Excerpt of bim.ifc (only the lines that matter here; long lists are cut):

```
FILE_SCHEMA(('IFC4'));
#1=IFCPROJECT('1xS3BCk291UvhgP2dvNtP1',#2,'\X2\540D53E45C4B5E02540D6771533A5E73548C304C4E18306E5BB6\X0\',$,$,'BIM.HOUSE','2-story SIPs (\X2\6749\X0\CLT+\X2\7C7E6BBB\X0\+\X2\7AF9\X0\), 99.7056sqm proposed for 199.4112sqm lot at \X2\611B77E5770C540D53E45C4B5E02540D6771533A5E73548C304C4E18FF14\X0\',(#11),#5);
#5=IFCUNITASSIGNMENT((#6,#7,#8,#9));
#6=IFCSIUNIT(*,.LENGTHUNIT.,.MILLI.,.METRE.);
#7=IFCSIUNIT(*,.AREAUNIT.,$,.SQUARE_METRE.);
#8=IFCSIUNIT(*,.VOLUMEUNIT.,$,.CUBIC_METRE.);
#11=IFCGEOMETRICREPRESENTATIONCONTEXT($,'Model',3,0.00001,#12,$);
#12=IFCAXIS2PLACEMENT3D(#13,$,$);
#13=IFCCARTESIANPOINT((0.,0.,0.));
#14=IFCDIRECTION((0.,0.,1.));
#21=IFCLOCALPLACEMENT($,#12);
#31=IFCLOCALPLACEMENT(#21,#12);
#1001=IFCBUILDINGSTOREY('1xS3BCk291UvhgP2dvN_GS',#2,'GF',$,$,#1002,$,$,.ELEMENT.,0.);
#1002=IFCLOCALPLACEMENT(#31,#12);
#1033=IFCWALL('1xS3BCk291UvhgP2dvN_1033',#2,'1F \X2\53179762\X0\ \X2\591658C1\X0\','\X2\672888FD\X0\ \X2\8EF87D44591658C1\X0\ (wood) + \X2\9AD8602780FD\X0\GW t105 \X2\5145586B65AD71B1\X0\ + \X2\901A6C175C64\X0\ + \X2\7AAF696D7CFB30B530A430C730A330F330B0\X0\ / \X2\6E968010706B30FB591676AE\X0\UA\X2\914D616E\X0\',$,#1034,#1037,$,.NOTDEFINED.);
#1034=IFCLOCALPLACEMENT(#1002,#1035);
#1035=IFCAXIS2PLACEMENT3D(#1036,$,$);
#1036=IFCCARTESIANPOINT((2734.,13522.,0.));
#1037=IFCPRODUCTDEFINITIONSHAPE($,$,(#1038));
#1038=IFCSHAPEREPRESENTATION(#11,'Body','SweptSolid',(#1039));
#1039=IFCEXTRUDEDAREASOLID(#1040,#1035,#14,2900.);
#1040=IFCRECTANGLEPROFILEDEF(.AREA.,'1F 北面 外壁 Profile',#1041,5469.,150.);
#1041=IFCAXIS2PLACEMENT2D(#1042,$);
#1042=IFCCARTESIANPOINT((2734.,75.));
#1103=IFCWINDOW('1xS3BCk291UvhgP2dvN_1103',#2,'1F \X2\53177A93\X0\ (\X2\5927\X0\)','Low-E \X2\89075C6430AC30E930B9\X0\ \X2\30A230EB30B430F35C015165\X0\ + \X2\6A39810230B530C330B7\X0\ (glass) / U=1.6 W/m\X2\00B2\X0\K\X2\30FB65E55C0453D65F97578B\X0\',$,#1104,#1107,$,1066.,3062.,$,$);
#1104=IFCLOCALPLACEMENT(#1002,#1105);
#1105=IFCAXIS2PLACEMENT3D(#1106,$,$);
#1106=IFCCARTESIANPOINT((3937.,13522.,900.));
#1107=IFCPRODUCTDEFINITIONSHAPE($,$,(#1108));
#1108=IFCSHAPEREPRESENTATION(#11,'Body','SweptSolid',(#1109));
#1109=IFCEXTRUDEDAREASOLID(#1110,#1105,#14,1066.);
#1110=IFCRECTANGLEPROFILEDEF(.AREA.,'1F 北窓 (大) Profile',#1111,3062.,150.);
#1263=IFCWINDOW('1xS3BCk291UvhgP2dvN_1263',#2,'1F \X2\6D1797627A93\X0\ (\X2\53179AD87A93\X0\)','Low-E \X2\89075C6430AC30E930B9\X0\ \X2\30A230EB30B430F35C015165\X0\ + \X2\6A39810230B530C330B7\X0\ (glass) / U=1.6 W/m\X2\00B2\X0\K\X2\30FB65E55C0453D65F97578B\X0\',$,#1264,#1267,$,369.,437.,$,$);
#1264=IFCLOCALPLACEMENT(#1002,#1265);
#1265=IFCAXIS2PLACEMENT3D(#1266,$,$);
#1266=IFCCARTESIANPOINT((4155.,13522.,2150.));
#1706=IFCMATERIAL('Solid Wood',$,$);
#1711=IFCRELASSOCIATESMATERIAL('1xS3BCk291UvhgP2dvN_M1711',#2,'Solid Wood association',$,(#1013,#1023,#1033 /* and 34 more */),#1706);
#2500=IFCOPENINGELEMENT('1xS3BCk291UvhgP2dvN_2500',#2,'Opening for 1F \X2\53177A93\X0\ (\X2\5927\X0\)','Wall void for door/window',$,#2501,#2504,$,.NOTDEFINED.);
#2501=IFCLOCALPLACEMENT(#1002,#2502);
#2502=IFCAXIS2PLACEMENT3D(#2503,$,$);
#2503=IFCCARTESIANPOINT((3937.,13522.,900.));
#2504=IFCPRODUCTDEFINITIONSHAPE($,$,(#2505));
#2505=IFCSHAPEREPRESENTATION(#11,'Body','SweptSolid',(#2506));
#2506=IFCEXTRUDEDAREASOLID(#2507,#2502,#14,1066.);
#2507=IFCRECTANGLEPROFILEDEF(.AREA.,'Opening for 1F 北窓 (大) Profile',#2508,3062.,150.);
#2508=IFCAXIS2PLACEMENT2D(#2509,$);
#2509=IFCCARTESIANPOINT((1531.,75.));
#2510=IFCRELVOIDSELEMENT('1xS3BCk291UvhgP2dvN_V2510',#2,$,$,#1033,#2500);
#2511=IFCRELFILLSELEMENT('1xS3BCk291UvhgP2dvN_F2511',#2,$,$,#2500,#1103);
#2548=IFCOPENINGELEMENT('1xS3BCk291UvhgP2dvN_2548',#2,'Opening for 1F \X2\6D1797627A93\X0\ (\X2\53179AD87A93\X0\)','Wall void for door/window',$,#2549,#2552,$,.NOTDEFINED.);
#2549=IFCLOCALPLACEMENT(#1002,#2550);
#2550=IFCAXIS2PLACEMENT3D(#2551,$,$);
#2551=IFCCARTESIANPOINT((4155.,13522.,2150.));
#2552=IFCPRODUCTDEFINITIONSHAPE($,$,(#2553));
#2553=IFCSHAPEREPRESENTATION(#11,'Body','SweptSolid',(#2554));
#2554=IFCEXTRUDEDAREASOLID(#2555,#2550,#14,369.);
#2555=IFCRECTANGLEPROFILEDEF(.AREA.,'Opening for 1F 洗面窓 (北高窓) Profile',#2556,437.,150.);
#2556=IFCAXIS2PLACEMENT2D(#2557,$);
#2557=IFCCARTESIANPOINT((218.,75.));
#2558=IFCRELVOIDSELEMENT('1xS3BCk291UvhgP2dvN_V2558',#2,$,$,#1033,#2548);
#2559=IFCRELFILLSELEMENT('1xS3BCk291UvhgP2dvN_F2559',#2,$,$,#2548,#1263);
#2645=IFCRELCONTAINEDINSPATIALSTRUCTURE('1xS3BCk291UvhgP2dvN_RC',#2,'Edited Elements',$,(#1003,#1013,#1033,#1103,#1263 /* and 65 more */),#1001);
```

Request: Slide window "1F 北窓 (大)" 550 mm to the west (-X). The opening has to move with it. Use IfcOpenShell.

```python
import ifcopenshell
import ifcopenshell.api.geometry
import ifcopenshell.util.placement

model = ifcopenshell.open("bim.ifc")

window = model.by_guid("1xS3BCk291UvhgP2dvN_1103")
opening = window.FillsVoids[0].RelatingOpeningElement
wall = opening.VoidsElements[0].RelatingBuildingElement

wall_matrix = ifcopenshell.util.placement.get_local_placement(wall.ObjectPlacement)
shift = wall_matrix[:3, 0] * -550.0
before = ifcopenshell.util.placement.get_local_placement(window.ObjectPlacement)[:3, 3].copy()

# The window is not placed relative to its opening, so move both.
for product in (opening, window):
    matrix = ifcopenshell.util.placement.get_local_placement(product.ObjectPlacement)
    matrix[:3, 3] += shift
    ifcopenshell.api.geometry.edit_object_placement(model, product=product, matrix=matrix, is_si=False)

after = ifcopenshell.util.placement.get_local_placement(window.ObjectPlacement)[:3, 3]
print("window moved by", (after - before).round(3) + 0.0)

model.write("bim_updated.ifc")
```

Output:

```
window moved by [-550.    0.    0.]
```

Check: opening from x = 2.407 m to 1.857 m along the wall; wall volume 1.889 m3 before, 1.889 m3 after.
